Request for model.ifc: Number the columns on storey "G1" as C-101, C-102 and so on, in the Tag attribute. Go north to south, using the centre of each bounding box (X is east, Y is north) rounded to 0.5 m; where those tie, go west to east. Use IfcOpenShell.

First a look at what the model holds.

```python
import ifcopenshell
import ifcopenshell.util.element
import ifcopenshell.util.placement

model = ifcopenshell.open("model.ifc")
print(model.schema)
storey = next(s for s in model.by_type("IfcBuildingStorey") if s.Name == "G1")
columns = [e for e in ifcopenshell.util.element.get_decomposition(storey) if e.is_a("IfcColumn")]
for e in sorted(columns, key=lambda e: e.id()):
    origin = ifcopenshell.util.placement.get_local_placement(e.ObjectPlacement)[:3, 3]
    print(e.id(), e.Tag, e.Name, origin.round(2) + 0.0, sep=" | ")
```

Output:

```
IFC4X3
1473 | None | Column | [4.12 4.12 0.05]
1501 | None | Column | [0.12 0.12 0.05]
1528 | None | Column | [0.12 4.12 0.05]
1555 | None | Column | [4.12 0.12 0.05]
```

```python
import ifcopenshell
import ifcopenshell.geom
import ifcopenshell.util.element
import ifcopenshell.util.shape

model = ifcopenshell.open("model.ifc")
settings = ifcopenshell.geom.settings()
settings.set("use-world-coords", True)


def centre(element):
    shape = ifcopenshell.geom.create_shape(settings, element)
    return ifcopenshell.util.shape.get_bbox_centroid(shape.geometry)


storey = next(s for s in model.by_type("IfcBuildingStorey") if s.Name == "G1")
columns = [e for e in ifcopenshell.util.element.get_decomposition(storey) if e.is_a("IfcColumn")]

# Insertion points can sit at a corner or the storey origin, so sort by the geometry (in metres).
centres = {e: centre(e) for e in columns}
columns.sort(key=lambda e: (-round(centres[e][1] / 0.5), centres[e][0]))

for i, e in enumerate(columns, start=1):
    number = f"C-1{i:02d}"
    e.Tag = number
    print(e.id(), number)

model.write("model_updated.ifc")
```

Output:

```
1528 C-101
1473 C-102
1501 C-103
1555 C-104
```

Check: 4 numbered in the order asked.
